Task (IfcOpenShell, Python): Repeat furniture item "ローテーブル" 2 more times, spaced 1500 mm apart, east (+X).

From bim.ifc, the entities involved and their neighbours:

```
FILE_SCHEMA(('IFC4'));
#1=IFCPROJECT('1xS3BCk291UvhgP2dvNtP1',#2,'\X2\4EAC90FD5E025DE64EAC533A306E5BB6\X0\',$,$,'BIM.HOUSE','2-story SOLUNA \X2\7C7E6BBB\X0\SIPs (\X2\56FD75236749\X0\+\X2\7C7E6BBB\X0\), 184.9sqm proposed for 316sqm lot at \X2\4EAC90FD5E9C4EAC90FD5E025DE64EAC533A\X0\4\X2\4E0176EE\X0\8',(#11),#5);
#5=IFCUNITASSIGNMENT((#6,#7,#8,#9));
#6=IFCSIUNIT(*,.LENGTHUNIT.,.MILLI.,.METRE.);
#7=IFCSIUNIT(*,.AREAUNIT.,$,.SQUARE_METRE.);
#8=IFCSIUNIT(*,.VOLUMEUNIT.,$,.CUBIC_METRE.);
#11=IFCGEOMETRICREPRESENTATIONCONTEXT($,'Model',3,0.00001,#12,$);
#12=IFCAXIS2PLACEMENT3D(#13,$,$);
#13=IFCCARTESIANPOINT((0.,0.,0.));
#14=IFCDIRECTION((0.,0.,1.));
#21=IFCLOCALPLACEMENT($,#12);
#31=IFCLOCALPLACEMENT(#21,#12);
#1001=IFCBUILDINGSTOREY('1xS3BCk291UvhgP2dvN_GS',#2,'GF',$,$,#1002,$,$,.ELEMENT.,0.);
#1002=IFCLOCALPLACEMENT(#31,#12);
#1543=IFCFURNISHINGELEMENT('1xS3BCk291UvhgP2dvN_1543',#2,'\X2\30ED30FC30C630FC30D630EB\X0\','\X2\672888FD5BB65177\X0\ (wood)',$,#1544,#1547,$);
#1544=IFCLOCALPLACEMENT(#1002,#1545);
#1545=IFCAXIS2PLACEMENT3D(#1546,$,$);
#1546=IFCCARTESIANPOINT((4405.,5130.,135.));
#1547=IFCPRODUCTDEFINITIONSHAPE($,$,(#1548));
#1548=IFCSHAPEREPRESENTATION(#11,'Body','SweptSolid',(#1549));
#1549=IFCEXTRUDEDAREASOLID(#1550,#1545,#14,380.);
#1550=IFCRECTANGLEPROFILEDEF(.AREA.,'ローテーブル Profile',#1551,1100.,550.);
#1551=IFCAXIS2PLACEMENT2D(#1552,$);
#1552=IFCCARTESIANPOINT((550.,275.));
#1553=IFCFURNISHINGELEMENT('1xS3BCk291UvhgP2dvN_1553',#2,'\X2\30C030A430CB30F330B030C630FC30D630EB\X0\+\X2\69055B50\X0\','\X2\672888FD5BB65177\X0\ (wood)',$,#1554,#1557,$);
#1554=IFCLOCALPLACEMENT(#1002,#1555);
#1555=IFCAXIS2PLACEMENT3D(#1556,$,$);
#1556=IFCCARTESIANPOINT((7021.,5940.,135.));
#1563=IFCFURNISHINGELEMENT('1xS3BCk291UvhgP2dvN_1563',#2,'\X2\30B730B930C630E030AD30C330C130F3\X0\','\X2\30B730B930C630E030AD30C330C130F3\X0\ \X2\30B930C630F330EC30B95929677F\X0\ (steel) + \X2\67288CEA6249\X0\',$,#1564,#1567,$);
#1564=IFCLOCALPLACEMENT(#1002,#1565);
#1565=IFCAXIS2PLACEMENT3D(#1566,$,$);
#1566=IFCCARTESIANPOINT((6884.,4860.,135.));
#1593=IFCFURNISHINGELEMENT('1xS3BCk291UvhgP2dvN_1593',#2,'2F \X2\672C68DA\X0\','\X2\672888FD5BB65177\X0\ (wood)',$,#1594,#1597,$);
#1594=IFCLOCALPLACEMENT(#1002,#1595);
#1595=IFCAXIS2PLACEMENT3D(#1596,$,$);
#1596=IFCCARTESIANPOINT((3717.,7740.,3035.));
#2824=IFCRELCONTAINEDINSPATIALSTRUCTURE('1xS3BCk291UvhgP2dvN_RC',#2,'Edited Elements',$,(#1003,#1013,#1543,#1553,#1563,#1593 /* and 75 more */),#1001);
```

```python
import numpy as np
import ifcopenshell
import ifcopenshell.api.geometry
import ifcopenshell.api.root
import ifcopenshell.util.element
import ifcopenshell.util.placement
import ifcopenshell.util.unit

model = ifcopenshell.open("bim.ifc")
unit_scale = ifcopenshell.util.unit.calculate_unit_scale(model)


def reuse_history(source, copy):
    """copy_class also copies each property set's owner history, people and application; keep the originals."""
    for rel in copy.IsDefinedBy:
        if rel.is_a("IfcRelDefinesByProperties") and (history := rel.RelatingPropertyDefinition.OwnerHistory):
            rel.RelatingPropertyDefinition.OwnerHistory = source.OwnerHistory
            ifcopenshell.util.element.remove_deep2(model, history)


source = model.by_guid("1xS3BCk291UvhgP2dvN_1543")
base = ifcopenshell.util.placement.get_local_placement(source.ObjectPlacement)
step = np.array([1.0, 0.0, 0.0]) * 1.5 / unit_scale

for i in range(1, 3):
    copy = ifcopenshell.api.root.copy_class(model, product=source)
    copy.Representation = ifcopenshell.util.element.copy_deep(
        model, source.Representation, exclude=["IfcGeometricRepresentationContext", "IfcRepresentationMap"]
    )
    reuse_history(source, copy)
    matrix = base.copy()
    matrix[:3, 3] += i * step
    print("added at", matrix[:3, 3].round(3) + 0.0)
    ifcopenshell.api.geometry.edit_object_placement(model, product=copy, matrix=matrix, is_si=False)

model.write("bim_v2.ifc")
```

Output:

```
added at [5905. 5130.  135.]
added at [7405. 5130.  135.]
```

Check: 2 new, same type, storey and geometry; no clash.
